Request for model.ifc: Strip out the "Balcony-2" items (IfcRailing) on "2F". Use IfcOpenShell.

First a look at what the model holds.

```python
import ifcopenshell
import ifcopenshell.util.element

model = ifcopenshell.open("model.ifc")
print(model.schema)
storey = next(s for s in model.by_type("IfcBuildingStorey") if s.Name == "2F")
railings = [e for e in ifcopenshell.util.element.get_decomposition(storey) if e.is_a("IfcRailing")]
seen = {}
for e in railings:
    element_type = ifcopenshell.util.element.get_type(e)
    name = element_type.Name if element_type not in (None, e) else None
    seen[name] = seen.get(name, 0) + 1
for name, count in sorted(seen.items(), key=str):
    print(count, "x", name)
```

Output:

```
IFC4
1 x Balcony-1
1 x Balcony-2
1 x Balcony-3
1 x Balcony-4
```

```python
import ifcopenshell
import ifcopenshell.api.root
import ifcopenshell.util.element

model = ifcopenshell.open("model.ifc")

storey = next(s for s in model.by_type("IfcBuildingStorey") if s.Name == "2F")
railings = [e for e in ifcopenshell.util.element.get_decomposition(storey) if e.is_a("IfcRailing")]
targets = [e for e in railings if (t := ifcopenshell.util.element.get_type(e)) not in (None, e) and t.Name == "Balcony-2"]

for e in targets:
    ifcopenshell.api.root.remove_product(model, product=e)
print(len(targets), "removed")

model.write("model_edited.ifc")
```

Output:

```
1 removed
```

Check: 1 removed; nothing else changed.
